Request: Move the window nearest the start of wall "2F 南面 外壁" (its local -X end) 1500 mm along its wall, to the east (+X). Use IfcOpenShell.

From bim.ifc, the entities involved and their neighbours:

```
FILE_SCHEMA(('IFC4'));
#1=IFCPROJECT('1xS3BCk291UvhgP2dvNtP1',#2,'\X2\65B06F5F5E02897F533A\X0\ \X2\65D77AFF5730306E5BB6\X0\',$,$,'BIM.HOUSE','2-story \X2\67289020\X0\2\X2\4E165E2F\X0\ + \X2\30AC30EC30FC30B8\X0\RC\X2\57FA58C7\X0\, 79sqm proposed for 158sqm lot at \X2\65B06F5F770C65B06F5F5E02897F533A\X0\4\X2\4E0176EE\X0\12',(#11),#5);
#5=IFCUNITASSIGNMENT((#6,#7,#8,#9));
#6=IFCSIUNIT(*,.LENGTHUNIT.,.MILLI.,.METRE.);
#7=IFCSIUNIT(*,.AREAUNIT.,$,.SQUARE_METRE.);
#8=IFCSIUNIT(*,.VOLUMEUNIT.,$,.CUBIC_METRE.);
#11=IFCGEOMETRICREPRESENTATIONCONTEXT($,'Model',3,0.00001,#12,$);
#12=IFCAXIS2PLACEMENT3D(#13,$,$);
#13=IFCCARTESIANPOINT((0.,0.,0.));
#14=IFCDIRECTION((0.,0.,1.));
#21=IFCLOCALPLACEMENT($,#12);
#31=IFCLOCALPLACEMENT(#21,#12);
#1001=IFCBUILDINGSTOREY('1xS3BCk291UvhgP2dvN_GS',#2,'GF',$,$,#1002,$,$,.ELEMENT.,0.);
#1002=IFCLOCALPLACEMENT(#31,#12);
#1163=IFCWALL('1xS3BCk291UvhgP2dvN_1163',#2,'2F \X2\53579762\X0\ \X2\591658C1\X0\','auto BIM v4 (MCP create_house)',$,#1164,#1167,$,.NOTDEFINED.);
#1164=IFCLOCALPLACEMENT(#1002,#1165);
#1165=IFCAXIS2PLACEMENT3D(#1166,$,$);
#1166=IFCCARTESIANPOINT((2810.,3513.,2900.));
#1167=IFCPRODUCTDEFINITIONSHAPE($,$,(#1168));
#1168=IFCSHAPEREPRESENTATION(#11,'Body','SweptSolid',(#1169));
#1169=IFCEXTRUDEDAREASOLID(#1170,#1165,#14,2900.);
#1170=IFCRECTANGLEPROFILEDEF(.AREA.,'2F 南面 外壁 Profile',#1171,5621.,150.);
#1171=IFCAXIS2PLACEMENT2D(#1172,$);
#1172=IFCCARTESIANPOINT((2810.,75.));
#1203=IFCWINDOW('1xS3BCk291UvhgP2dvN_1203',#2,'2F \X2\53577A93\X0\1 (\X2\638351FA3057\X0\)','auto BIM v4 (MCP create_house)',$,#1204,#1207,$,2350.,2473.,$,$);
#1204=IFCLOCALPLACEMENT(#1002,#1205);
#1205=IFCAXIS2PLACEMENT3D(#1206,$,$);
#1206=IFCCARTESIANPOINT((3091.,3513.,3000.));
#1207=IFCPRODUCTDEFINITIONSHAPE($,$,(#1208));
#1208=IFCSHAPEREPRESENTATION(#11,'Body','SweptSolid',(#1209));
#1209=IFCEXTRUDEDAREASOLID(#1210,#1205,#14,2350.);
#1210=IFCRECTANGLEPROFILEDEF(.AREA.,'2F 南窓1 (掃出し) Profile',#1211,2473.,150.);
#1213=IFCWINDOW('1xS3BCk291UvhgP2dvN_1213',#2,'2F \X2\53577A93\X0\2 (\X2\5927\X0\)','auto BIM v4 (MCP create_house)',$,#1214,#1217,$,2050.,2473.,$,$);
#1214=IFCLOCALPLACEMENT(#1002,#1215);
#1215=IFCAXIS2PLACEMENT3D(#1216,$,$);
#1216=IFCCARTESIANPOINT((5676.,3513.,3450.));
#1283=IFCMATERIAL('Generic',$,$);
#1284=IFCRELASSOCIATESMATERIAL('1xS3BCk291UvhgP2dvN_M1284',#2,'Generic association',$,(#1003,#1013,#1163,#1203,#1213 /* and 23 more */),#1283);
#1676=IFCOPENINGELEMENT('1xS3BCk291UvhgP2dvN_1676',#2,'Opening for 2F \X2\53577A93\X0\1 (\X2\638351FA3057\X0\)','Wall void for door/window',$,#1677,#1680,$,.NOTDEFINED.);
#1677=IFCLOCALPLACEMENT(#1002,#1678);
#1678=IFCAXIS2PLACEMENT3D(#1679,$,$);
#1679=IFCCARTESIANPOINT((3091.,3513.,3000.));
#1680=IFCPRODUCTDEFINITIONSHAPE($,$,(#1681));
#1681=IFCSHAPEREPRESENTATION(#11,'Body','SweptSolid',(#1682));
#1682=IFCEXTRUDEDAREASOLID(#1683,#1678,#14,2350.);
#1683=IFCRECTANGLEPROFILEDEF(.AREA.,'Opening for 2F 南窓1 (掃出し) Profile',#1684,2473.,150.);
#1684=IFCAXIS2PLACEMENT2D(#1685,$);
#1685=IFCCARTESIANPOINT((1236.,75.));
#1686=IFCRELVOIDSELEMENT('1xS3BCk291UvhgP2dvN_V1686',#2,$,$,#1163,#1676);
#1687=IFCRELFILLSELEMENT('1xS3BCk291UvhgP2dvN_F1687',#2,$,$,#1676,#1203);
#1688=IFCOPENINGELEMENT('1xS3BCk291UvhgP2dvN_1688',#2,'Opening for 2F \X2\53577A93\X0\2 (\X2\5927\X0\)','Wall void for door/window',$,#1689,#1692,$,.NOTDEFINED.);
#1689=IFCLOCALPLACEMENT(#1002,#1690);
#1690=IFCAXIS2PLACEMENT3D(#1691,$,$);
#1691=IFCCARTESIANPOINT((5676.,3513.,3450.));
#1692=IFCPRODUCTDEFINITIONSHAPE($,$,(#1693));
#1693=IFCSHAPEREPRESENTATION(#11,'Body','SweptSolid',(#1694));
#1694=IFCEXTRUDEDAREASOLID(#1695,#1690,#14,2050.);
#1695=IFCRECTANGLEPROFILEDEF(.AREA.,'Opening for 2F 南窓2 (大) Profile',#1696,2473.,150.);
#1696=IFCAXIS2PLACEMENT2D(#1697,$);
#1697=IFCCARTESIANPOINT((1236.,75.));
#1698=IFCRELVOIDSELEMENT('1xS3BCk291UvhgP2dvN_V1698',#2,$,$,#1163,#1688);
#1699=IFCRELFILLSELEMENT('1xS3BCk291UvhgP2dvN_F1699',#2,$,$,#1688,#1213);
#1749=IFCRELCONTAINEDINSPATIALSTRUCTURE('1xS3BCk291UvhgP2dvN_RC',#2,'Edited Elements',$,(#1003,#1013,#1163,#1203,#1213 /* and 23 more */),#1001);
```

```python
import ifcopenshell
import ifcopenshell.api.geometry
import ifcopenshell.util.placement
import ifcopenshell.util.unit

model = ifcopenshell.open("bim.ifc")
unit_scale = ifcopenshell.util.unit.calculate_unit_scale(model)

window = model.by_guid("1xS3BCk291UvhgP2dvN_1203")
opening = window.FillsVoids[0].RelatingOpeningElement
wall = opening.VoidsElements[0].RelatingBuildingElement

wall_matrix = ifcopenshell.util.placement.get_local_placement(wall.ObjectPlacement)
shift = wall_matrix[:3, 0] * 1.5 / unit_scale
before = ifcopenshell.util.placement.get_local_placement(window.ObjectPlacement)[:3, 3].copy()

# The window is not placed relative to its opening, so move both.
for product in (opening, window):
    matrix = ifcopenshell.util.placement.get_local_placement(product.ObjectPlacement)
    matrix[:3, 3] += shift
    ifcopenshell.api.geometry.edit_object_placement(model, product=product, matrix=matrix, is_si=False)

after = ifcopenshell.util.placement.get_local_placement(window.ObjectPlacement)[:3, 3]
print("window moved by", (after - before).round(3) + 0.0)

model.write("bim_edited.ifc")
```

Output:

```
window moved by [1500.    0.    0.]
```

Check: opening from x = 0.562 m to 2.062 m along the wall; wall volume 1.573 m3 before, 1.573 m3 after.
